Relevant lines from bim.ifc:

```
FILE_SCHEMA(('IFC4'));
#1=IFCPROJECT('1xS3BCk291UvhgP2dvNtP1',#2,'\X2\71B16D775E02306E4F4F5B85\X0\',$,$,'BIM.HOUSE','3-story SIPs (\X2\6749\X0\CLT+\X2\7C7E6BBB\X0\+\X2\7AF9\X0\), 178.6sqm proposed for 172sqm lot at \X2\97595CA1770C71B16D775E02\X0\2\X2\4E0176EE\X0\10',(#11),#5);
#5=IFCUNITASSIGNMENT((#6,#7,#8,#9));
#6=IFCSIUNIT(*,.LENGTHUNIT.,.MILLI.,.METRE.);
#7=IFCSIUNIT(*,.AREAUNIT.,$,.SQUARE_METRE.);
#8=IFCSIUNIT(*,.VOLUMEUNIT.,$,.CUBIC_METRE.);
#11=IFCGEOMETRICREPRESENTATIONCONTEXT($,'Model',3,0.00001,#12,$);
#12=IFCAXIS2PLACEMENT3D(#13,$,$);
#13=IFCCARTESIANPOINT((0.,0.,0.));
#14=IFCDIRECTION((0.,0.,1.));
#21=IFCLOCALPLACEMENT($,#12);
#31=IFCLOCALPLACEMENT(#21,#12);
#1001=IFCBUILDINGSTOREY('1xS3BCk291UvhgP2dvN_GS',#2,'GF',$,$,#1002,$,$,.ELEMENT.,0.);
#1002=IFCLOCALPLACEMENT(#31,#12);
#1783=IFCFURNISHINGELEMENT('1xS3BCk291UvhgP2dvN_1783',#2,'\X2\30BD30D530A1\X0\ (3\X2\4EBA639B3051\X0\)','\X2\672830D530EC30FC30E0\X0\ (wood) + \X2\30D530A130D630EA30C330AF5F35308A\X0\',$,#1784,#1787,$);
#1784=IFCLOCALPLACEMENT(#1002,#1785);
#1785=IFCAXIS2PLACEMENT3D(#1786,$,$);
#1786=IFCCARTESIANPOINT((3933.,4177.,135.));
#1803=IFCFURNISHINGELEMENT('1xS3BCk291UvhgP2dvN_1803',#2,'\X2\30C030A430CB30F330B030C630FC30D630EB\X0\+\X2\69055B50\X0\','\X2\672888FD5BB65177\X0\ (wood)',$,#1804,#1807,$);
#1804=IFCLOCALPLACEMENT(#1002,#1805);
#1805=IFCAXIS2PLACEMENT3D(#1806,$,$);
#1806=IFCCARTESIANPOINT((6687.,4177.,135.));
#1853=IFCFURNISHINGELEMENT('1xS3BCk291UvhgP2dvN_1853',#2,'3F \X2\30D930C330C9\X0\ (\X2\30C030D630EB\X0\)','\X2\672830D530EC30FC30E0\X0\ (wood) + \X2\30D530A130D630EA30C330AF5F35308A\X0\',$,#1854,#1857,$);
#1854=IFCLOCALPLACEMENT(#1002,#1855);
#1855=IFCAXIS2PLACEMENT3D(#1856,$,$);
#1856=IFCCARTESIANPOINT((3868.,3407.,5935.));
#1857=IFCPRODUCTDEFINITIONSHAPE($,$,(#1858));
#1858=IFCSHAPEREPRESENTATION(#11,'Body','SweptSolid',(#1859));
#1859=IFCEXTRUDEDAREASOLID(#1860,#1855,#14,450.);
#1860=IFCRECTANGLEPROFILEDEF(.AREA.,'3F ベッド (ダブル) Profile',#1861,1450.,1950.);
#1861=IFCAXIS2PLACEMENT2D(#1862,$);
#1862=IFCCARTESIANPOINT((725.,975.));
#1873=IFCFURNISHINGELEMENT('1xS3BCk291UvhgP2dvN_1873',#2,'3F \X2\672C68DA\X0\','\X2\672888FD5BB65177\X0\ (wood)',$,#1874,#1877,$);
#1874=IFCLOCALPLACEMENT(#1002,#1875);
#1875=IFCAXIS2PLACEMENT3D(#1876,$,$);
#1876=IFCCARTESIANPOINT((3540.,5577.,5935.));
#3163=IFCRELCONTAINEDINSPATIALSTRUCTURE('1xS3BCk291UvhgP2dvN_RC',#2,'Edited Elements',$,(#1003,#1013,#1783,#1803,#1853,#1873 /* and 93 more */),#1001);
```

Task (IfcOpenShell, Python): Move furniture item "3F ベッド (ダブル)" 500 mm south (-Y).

```python
import ifcopenshell
import ifcopenshell.api.geometry
import ifcopenshell.util.placement

model = ifcopenshell.open("bim.ifc")

item = model.by_guid("1xS3BCk291UvhgP2dvN_1853")
matrix = ifcopenshell.util.placement.get_local_placement(item.ObjectPlacement)
matrix[1, 3] -= 500.0
ifcopenshell.api.geometry.edit_object_placement(model, product=item, matrix=matrix, is_si=False)

print(ifcopenshell.util.placement.get_local_placement(item.ObjectPlacement).round(3) + 0.0)

model.write("bim_updated.ifc")
```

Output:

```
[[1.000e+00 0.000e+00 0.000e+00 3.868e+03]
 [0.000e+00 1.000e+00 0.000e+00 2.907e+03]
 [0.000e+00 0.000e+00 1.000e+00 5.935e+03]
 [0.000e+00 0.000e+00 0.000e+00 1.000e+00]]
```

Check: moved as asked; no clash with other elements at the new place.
